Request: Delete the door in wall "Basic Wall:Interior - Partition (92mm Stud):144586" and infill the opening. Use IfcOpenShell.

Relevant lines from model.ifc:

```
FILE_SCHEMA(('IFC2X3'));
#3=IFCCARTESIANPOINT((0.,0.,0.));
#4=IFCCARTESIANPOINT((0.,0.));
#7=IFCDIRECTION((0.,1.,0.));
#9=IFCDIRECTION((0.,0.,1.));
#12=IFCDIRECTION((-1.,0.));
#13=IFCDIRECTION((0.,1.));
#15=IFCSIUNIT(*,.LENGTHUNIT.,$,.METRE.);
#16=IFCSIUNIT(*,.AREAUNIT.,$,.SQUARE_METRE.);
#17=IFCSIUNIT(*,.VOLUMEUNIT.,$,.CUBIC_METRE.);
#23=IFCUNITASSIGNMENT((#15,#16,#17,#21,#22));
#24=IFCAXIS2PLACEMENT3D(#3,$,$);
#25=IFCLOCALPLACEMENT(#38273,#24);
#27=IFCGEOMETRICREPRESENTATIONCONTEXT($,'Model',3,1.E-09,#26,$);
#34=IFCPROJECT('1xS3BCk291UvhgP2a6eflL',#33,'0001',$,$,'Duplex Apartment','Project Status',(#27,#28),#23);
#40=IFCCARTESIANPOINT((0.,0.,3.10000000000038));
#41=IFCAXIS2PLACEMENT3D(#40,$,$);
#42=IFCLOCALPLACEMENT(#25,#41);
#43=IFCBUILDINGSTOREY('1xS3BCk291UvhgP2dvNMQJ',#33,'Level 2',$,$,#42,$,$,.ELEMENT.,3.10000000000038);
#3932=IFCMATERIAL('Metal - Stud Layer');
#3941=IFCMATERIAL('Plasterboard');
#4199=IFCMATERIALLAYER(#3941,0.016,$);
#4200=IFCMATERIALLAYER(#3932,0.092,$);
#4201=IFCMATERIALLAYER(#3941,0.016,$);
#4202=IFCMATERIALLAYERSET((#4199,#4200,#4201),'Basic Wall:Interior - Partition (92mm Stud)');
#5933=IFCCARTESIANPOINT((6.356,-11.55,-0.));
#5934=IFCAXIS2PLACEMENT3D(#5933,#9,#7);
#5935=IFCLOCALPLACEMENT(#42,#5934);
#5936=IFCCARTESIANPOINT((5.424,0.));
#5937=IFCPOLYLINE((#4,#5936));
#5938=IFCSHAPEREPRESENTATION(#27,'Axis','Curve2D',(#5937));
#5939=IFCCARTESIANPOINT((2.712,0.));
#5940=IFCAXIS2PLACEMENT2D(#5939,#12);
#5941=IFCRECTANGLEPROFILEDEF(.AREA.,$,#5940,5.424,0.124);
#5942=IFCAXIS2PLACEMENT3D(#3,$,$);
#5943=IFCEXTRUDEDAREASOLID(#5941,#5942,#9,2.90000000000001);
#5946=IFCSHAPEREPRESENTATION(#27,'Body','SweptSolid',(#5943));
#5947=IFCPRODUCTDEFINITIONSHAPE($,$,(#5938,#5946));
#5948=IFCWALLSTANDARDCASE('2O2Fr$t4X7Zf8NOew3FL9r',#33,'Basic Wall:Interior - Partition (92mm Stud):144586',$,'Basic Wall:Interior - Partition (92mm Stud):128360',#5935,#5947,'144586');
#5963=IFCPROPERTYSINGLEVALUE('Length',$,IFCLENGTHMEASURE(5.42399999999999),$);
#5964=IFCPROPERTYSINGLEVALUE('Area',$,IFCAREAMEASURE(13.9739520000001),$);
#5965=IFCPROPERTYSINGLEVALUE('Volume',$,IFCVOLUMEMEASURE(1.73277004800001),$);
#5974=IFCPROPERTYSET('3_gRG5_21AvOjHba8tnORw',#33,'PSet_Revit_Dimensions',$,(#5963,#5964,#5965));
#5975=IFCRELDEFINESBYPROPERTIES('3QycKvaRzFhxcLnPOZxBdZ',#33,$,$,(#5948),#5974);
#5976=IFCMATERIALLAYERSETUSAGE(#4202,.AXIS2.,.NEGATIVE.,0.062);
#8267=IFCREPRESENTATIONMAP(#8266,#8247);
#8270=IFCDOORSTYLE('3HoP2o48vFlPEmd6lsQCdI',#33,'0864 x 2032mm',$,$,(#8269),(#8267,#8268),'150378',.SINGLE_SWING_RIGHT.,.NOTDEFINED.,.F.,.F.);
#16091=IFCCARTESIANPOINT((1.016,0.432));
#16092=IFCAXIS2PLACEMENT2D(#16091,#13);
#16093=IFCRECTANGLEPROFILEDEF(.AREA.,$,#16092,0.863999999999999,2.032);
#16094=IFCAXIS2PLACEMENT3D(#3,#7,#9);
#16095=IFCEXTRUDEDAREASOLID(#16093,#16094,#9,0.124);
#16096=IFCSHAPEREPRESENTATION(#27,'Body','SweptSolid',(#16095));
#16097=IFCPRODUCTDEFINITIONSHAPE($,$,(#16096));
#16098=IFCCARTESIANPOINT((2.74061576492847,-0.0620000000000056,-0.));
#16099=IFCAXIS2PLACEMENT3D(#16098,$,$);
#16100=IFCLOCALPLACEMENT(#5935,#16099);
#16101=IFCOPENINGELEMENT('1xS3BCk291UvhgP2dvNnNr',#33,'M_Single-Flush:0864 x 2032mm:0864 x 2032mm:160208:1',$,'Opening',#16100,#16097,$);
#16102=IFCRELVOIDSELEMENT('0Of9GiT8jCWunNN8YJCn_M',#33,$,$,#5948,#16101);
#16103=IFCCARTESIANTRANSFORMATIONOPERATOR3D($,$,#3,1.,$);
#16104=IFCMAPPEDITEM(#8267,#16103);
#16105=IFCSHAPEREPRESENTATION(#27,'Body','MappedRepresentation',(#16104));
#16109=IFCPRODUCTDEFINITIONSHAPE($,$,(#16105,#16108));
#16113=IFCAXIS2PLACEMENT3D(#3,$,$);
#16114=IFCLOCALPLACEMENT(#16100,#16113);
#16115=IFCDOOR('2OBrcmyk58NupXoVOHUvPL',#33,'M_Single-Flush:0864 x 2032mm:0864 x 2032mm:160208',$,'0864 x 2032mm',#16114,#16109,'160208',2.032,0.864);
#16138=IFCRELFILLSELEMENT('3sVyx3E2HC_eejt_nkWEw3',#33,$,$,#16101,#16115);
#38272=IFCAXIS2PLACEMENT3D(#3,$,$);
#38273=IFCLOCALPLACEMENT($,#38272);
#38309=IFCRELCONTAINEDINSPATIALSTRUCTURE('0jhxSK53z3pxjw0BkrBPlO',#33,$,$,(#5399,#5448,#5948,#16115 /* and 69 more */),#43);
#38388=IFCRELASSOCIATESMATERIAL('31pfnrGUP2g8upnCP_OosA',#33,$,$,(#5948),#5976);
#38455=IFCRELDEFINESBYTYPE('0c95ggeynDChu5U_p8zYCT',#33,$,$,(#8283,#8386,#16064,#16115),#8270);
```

```python
import ifcopenshell
import ifcopenshell.api.feature
import ifcopenshell.api.pset
import ifcopenshell.api.root
import ifcopenshell.geom
import ifcopenshell.util.element
import ifcopenshell.util.shape
import ifcopenshell.util.unit

model = ifcopenshell.open("model.ifc")
area_scale = ifcopenshell.util.unit.calculate_unit_scale(model, "AREAUNIT")
volume_scale = ifcopenshell.util.unit.calculate_unit_scale(model, "VOLUMEUNIT")
settings = ifcopenshell.geom.settings()


def volume(element):
    """Net volume in cubic metres, openings subtracted."""
    shape = ifcopenshell.geom.create_shape(settings, element)
    return ifcopenshell.util.shape.get_volume(shape.geometry)


door = model.by_guid("2OBrcmyk58NupXoVOHUvPL")
opening = door.FillsVoids[0].RelatingOpeningElement
wall = opening.VoidsElements[0].RelatingBuildingElement
before = volume(wall)

ifcopenshell.api.root.remove_product(model, product=door)
ifcopenshell.api.feature.remove_feature(model, feature=opening)

after = volume(wall)
thickness = 0.124  # wall thickness in metres

# Update the wall's stored quantities.
pset = model.by_id(ifcopenshell.util.element.get_pset(wall, "PSet_Revit_Dimensions", should_inherit=False)["id"])
ifcopenshell.api.pset.edit_pset(model, pset=pset, properties={
    "Area": model.create_entity("IfcAreaMeasure", after / thickness / area_scale),
    "Volume": model.create_entity("IfcVolumeMeasure", after / volume_scale),
})

print(f"wall volume {before:.3f} -> {after:.3f} m3")

model.write("model_edited.ifc")
```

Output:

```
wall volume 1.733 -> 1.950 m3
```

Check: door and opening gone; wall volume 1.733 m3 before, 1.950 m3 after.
